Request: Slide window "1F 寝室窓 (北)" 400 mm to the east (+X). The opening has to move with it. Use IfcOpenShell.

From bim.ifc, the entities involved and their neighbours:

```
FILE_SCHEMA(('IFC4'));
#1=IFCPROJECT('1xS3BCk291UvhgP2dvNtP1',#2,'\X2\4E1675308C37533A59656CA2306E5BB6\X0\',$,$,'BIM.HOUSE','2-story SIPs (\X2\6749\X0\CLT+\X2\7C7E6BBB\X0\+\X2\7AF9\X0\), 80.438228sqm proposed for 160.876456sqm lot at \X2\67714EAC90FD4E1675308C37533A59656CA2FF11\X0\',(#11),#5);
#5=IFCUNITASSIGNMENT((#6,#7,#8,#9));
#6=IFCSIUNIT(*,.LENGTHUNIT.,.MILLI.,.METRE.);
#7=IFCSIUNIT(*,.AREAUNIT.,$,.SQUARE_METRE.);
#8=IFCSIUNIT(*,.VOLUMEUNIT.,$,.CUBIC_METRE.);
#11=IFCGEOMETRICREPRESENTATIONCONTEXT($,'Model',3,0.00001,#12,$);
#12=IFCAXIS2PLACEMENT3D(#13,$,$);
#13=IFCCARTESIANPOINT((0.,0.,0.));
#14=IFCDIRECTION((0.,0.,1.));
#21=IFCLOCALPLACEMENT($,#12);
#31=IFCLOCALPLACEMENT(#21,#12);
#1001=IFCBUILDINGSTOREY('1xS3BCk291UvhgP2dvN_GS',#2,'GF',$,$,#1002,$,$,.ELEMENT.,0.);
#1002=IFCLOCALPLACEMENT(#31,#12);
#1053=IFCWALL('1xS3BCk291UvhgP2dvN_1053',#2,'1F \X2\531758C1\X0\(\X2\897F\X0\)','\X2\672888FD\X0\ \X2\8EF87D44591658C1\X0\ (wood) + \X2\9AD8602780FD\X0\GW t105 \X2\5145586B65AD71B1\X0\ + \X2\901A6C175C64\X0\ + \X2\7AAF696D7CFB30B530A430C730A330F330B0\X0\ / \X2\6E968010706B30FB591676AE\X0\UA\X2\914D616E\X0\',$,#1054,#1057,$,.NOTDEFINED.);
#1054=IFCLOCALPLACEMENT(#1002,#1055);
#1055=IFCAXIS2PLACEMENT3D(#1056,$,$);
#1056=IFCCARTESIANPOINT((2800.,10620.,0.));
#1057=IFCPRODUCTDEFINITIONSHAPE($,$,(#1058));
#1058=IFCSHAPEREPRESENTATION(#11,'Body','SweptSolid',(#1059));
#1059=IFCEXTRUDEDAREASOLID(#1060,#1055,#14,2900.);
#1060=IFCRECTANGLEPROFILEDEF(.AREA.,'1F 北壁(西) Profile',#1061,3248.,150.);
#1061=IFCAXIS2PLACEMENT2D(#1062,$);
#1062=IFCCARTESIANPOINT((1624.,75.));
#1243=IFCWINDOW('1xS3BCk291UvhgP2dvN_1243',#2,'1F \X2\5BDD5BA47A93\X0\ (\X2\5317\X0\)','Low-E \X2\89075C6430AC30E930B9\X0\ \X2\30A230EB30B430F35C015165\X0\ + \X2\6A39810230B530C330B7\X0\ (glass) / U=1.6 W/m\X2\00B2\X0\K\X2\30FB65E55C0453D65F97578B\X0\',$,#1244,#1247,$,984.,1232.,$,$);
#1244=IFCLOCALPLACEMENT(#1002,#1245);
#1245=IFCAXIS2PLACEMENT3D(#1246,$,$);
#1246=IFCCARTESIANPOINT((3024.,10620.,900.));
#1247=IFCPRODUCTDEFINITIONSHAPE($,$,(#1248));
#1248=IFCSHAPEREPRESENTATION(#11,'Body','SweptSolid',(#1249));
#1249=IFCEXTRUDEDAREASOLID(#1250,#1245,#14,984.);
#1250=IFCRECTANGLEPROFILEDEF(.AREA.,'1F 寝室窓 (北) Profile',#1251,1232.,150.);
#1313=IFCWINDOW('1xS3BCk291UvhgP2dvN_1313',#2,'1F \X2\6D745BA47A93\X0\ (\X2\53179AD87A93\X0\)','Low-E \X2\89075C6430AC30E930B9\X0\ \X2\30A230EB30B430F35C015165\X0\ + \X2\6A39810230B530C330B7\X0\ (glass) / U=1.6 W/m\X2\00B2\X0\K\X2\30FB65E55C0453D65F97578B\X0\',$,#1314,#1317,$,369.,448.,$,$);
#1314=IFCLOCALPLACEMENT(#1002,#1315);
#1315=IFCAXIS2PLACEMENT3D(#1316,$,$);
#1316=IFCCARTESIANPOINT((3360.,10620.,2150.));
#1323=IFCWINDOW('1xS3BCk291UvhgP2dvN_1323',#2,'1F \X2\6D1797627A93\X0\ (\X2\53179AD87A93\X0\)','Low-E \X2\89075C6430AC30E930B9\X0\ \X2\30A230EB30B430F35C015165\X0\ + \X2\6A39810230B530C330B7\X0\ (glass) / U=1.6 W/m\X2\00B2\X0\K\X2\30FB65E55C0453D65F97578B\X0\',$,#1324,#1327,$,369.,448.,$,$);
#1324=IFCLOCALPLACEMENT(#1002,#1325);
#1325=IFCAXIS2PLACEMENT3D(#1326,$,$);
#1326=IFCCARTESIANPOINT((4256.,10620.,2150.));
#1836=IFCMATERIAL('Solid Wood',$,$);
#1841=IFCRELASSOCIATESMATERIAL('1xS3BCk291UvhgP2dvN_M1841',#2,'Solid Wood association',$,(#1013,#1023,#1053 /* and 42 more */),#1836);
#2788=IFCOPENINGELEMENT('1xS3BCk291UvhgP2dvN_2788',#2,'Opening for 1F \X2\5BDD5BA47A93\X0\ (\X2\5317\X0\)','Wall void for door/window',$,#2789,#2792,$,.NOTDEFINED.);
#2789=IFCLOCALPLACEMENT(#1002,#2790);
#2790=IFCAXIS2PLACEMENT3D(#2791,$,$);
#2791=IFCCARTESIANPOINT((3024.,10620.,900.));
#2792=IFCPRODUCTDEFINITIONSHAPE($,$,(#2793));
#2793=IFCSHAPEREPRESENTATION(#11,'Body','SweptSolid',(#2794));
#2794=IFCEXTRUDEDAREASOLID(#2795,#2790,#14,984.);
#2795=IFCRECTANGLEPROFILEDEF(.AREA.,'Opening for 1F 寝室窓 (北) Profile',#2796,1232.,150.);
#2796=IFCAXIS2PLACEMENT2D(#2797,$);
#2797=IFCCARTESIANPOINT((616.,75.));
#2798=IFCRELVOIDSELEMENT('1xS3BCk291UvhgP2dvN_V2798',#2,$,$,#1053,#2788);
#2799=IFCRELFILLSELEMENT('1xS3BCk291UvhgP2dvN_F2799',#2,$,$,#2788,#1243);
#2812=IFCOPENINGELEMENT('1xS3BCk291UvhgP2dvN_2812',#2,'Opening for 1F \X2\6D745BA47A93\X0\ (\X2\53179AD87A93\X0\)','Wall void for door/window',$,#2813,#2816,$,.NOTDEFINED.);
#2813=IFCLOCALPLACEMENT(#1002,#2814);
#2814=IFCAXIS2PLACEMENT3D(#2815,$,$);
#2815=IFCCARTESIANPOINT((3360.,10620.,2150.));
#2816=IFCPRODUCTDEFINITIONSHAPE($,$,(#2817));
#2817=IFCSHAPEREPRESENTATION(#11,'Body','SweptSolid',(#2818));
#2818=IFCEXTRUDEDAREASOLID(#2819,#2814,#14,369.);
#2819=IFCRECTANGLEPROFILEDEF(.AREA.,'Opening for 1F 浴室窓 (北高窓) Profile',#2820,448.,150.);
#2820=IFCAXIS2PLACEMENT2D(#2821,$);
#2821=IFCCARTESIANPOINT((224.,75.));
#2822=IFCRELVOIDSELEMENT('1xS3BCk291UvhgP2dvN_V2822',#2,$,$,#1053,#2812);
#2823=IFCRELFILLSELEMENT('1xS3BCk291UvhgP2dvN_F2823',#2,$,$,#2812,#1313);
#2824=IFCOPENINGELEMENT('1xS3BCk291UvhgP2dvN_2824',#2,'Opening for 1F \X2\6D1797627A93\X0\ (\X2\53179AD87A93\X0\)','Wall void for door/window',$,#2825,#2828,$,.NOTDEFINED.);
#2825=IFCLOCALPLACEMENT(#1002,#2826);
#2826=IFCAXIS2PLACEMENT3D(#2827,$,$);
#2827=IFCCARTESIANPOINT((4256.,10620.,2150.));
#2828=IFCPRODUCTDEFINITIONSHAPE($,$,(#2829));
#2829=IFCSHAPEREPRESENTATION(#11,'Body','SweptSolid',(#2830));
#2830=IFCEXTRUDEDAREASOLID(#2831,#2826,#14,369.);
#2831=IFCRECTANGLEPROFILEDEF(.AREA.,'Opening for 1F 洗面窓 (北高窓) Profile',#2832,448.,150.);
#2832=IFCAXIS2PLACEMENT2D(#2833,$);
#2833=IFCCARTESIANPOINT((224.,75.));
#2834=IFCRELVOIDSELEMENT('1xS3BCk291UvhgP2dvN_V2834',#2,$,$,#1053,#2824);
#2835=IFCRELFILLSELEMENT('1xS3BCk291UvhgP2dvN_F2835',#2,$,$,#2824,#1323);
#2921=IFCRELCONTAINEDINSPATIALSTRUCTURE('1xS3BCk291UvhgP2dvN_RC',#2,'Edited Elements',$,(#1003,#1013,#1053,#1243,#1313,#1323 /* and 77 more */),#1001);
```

```python
import ifcopenshell
import ifcopenshell.api.geometry
import ifcopenshell.util.placement
import ifcopenshell.util.unit

model = ifcopenshell.open("bim.ifc")
unit_scale = ifcopenshell.util.unit.calculate_unit_scale(model)

window = model.by_guid("1xS3BCk291UvhgP2dvN_1243")
opening = window.FillsVoids[0].RelatingOpeningElement
wall = opening.VoidsElements[0].RelatingBuildingElement

wall_matrix = ifcopenshell.util.placement.get_local_placement(wall.ObjectPlacement)
shift = wall_matrix[:3, 0] * 0.4 / unit_scale
before = ifcopenshell.util.placement.get_local_placement(window.ObjectPlacement)[:3, 3].copy()

# The window is not placed relative to its opening, so move both.
for product in (opening, window):
    matrix = ifcopenshell.util.placement.get_local_placement(product.ObjectPlacement)
    matrix[:3, 3] += shift
    ifcopenshell.api.geometry.edit_object_placement(model, product=product, matrix=matrix, is_si=False)

after = ifcopenshell.util.placement.get_local_placement(window.ObjectPlacement)[:3, 3]
print("window moved by", (after - before).round(3) + 0.0)

model.write("bim_edited.ifc")
```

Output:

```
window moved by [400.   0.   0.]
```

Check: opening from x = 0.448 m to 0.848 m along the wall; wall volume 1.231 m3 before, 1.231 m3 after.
